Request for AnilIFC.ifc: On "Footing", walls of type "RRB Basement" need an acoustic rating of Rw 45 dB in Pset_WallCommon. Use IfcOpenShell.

First a look at what the model holds.

```python
import ifcopenshell
import ifcopenshell.util.element

model = ifcopenshell.open("AnilIFC.ifc")
print(model.schema)
storey = next(s for s in model.by_type("IfcBuildingStorey") if s.Name == "Footing")
walls = [e for e in ifcopenshell.util.element.get_decomposition(storey) if e.is_a("IfcWall")]
seen = {}
for e in walls:
    element_type = ifcopenshell.util.element.get_type(e)
    key = (element_type.Name if element_type != e and element_type else None, ifcopenshell.util.element.get_pset(e, "Pset_WallCommon", "AcousticRating"))
    seen[key] = seen.get(key, 0) + 1
for (name, value), count in sorted(seen.items(), key=str):
    print(count, "x", name, "|", value)
```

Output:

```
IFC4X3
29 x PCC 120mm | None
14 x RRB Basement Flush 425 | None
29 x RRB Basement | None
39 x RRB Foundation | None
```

```python
import ifcopenshell
import ifcopenshell.api.pset
import ifcopenshell.util.element

model = ifcopenshell.open("AnilIFC.ifc")

storey = next(s for s in model.by_type("IfcBuildingStorey") if s.Name == "Footing")
walls = [e for e in ifcopenshell.util.element.get_decomposition(storey) if e.is_a("IfcWall")]

count = 0
for e in walls:
    element_type = ifcopenshell.util.element.get_type(e)
    if element_type in (None, e) or element_type.Name != "RRB Basement":
        continue
    # add_pset returns the element's existing set when there is one.
    pset = ifcopenshell.api.pset.add_pset(model, product=e, name="Pset_WallCommon")
    ifcopenshell.api.pset.edit_pset(model, pset=pset, properties={"AcousticRating": "Rw 45 dB"})
    count += 1

print(count, "walls updated")

model.write("AnilIFC_rev.ifc")
```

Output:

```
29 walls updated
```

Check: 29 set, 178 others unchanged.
